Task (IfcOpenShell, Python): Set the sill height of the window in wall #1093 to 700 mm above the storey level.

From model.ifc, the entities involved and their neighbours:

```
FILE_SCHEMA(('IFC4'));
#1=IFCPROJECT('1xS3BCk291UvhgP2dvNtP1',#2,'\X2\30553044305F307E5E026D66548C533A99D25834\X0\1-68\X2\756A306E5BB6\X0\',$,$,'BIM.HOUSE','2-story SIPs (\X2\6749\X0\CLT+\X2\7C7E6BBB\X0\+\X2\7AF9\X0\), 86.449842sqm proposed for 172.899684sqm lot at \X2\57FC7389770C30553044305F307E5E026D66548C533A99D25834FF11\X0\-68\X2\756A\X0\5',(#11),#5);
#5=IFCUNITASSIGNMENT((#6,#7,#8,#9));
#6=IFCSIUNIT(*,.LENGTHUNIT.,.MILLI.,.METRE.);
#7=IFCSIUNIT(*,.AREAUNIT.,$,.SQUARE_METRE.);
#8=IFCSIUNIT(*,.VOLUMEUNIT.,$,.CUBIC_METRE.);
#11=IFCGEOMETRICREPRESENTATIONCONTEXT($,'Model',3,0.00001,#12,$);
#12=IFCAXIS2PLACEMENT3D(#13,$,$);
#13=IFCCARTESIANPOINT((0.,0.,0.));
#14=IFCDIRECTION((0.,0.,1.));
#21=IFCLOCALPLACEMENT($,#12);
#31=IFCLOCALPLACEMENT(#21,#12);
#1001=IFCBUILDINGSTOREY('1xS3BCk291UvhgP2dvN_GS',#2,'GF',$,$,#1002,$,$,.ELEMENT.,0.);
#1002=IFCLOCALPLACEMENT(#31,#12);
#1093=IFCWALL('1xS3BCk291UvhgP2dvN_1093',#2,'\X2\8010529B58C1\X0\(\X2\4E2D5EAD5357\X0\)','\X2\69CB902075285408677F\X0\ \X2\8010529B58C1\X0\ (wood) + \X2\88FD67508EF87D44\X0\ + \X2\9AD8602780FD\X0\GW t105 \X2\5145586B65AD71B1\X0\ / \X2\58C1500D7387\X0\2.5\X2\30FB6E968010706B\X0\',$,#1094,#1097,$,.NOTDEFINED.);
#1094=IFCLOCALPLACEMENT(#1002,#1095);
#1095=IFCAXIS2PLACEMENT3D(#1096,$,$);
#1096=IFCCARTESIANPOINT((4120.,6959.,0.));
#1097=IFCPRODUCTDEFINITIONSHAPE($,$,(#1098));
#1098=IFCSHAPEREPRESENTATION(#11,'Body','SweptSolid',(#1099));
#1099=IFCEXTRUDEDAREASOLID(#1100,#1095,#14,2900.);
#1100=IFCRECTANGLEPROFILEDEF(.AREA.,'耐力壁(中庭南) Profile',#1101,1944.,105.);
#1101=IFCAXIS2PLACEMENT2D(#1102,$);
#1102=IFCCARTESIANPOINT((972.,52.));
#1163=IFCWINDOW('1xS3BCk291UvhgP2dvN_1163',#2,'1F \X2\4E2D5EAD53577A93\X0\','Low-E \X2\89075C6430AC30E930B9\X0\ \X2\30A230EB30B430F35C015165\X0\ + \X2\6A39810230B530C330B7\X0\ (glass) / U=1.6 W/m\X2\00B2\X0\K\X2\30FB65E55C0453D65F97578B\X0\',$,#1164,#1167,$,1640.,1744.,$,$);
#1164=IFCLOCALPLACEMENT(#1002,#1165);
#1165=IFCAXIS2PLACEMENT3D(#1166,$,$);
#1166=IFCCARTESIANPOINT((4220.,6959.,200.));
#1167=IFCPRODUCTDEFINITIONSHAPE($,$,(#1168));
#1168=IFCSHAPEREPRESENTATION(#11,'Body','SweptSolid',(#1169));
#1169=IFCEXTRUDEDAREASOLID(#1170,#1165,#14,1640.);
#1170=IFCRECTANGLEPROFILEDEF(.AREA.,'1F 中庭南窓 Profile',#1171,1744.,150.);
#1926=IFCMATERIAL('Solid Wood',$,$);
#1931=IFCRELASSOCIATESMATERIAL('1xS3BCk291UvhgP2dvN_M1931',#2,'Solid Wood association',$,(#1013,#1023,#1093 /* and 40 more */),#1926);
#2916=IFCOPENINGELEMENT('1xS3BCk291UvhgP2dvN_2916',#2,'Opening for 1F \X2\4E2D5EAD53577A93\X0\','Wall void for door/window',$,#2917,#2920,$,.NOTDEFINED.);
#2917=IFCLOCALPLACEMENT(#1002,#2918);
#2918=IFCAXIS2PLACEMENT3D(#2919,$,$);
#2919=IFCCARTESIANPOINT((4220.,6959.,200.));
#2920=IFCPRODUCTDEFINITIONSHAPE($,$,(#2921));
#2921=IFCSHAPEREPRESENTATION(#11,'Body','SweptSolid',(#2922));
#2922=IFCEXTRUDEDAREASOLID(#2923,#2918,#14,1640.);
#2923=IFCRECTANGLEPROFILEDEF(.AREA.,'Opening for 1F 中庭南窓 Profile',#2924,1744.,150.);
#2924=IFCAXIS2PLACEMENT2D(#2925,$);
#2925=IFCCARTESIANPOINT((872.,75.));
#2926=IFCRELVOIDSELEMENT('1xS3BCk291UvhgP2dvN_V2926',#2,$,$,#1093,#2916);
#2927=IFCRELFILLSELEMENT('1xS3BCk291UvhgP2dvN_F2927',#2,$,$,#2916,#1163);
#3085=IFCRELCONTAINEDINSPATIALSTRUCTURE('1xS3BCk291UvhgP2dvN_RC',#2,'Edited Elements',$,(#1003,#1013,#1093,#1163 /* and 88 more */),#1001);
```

```python
import numpy as np
import ifcopenshell
import ifcopenshell.api.geometry
import ifcopenshell.geom
import ifcopenshell.util.element
import ifcopenshell.util.placement
import ifcopenshell.util.shape
import ifcopenshell.util.unit

model = ifcopenshell.open("model.ifc")
unit_scale = ifcopenshell.util.unit.calculate_unit_scale(model)

window = model.by_id(1163)
opening = window.FillsVoids[0].RelatingOpeningElement
storey = ifcopenshell.util.element.get_container(window, ifc_class="IfcBuildingStorey")
level = ifcopenshell.util.placement.get_local_placement(storey.ObjectPlacement)[2, 3]

# The opening's origin need not be at the sill, so measure its lowest point.
shape = ifcopenshell.geom.create_shape(ifcopenshell.geom.settings(), opening)
bottom = ifcopenshell.util.shape.get_shape_bottom_elevation(shape, shape.geometry) / unit_scale
dz = level + 700.0 - bottom

shift = np.array([0.0, 0.0, dz])
# The window is not placed relative to its opening, so move both.
for product in (opening, window):
    matrix = ifcopenshell.util.placement.get_local_placement(product.ObjectPlacement)
    matrix[:3, 3] += shift
    ifcopenshell.api.geometry.edit_object_placement(model, product=product, matrix=matrix, is_si=False)

print(f"moved by {dz * unit_scale:+.3f} m")

model.write("model_v2.ifc")
```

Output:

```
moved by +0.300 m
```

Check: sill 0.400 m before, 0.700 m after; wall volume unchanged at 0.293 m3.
